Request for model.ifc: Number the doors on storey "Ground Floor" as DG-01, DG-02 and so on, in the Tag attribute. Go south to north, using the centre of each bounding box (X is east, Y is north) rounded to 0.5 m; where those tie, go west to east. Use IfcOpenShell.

First a look at what the model holds.

```python
import ifcopenshell
import ifcopenshell.util.element
import ifcopenshell.util.placement

model = ifcopenshell.open("model.ifc")
print(model.schema)
storey = next(s for s in model.by_type("IfcBuildingStorey") if s.Name == "Ground Floor")
doors = [e for e in ifcopenshell.util.element.get_decomposition(storey) if e.is_a("IfcDoor")]
for e in sorted(doors, key=lambda e: e.id()):
    origin = ifcopenshell.util.placement.get_local_placement(e.ObjectPlacement)[:3, 3]
    print(e.id(), e.Tag, e.Name, origin.round(2) + 0.0, sep=" | ")
```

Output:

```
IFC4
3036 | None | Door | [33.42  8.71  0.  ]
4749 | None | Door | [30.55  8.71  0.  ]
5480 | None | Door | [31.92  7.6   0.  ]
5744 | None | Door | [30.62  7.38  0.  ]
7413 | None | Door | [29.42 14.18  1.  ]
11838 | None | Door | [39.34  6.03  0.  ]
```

```python
import ifcopenshell
import ifcopenshell.geom
import ifcopenshell.util.element
import ifcopenshell.util.shape

model = ifcopenshell.open("model.ifc")
settings = ifcopenshell.geom.settings()
settings.set("use-world-coords", True)


def centre(element):
    shape = ifcopenshell.geom.create_shape(settings, element)
    return ifcopenshell.util.shape.get_bbox_centroid(shape.geometry)


storey = next(s for s in model.by_type("IfcBuildingStorey") if s.Name == "Ground Floor")
doors = [e for e in ifcopenshell.util.element.get_decomposition(storey) if e.is_a("IfcDoor")]

# Insertion points can sit at a corner or the storey origin, so sort by the geometry (in metres).
centres = {e: centre(e) for e in doors}
doors.sort(key=lambda e: (round(centres[e][1] / 0.5), centres[e][0]))

for i, e in enumerate(doors, start=1):
    number = f"DG-{i:02d}"
    e.Tag = number
    print(e.id(), number)

model.write("model-out.ifc")
```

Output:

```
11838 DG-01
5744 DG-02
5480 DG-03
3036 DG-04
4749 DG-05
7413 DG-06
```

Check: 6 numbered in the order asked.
